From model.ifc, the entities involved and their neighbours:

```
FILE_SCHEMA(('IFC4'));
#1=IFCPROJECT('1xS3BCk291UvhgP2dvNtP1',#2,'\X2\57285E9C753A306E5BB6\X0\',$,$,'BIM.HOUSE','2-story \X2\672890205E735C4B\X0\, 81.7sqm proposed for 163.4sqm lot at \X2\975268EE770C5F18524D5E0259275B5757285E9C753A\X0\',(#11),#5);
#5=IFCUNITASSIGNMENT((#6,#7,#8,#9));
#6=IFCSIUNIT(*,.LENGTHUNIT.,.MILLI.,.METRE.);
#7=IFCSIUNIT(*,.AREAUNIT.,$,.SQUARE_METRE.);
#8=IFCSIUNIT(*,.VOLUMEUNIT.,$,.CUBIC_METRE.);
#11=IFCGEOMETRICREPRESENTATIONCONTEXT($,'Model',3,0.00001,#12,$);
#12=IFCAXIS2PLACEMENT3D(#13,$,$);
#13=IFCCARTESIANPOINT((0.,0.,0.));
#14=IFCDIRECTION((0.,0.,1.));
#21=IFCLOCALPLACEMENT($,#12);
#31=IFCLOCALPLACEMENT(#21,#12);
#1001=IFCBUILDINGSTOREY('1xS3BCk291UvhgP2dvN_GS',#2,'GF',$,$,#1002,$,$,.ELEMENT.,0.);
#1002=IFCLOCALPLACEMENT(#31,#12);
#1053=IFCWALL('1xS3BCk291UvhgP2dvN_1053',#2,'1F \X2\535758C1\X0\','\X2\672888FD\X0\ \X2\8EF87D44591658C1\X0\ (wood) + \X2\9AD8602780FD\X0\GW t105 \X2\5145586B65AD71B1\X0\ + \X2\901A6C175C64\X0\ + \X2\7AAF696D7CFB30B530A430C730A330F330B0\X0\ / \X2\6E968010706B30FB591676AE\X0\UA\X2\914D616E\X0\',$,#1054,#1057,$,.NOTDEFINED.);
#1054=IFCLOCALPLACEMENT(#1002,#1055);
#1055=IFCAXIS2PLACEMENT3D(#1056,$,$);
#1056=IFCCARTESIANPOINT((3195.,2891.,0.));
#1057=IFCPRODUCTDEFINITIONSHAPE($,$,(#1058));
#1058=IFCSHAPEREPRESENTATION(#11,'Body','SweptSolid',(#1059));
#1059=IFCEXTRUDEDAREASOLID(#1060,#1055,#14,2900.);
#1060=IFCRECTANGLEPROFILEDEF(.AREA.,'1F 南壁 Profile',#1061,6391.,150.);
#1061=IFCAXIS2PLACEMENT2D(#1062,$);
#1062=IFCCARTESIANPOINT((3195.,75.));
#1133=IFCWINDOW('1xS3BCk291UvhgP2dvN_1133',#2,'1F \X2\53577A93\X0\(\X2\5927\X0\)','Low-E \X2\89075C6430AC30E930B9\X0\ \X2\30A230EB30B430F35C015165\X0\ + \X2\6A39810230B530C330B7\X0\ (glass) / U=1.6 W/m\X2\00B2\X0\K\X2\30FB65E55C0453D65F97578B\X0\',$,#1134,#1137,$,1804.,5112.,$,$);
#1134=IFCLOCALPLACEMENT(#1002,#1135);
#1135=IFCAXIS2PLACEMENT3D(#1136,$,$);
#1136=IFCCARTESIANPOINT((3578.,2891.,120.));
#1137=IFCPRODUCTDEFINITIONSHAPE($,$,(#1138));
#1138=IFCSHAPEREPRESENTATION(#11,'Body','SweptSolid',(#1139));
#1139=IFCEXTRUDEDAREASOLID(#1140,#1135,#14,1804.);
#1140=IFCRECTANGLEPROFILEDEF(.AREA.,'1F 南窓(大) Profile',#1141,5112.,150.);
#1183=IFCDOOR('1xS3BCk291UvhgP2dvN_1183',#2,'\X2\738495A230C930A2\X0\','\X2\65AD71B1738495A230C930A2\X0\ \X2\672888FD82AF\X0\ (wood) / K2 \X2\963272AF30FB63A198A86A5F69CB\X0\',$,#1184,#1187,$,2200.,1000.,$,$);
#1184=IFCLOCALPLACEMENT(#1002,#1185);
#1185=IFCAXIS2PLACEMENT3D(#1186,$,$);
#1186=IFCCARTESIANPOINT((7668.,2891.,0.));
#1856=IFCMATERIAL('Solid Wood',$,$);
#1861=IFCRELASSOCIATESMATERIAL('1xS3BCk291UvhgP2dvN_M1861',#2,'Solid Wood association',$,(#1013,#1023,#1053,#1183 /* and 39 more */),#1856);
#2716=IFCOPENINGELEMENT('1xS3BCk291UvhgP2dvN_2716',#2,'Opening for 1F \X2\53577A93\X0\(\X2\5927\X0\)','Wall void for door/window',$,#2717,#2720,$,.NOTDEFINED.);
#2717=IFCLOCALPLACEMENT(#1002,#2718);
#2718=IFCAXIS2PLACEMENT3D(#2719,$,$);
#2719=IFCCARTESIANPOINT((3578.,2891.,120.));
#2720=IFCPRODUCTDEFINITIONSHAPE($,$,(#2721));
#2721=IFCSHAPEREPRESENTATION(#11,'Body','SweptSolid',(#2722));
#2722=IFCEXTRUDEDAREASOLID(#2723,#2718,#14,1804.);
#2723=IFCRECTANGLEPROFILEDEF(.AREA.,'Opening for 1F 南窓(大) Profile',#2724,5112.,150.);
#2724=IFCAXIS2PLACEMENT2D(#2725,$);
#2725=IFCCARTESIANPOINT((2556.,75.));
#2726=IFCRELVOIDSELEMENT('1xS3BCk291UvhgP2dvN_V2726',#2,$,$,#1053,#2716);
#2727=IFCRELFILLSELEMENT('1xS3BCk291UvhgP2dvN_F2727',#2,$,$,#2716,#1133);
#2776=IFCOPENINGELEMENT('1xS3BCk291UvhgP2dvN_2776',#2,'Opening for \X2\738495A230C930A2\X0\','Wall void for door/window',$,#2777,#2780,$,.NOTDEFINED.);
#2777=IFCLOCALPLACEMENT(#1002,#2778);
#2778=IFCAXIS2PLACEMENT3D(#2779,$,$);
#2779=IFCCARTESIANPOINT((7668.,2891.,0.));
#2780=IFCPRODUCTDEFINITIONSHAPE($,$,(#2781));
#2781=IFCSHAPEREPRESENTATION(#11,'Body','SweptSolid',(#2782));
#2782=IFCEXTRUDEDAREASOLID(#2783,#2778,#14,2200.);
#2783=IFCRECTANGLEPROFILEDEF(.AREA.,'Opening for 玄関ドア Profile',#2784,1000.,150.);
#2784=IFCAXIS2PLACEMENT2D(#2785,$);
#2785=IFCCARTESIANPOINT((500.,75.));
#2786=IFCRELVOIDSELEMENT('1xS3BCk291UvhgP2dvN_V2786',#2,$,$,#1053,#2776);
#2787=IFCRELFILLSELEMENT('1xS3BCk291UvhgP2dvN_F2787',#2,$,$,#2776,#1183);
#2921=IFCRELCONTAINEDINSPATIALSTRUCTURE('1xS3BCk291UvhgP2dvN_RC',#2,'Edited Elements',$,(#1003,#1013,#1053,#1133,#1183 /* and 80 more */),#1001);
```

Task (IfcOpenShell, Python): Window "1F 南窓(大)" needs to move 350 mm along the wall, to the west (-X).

```python
import ifcopenshell
import ifcopenshell.api.geometry
import ifcopenshell.util.placement
import ifcopenshell.util.unit

model = ifcopenshell.open("model.ifc")
unit_scale = ifcopenshell.util.unit.calculate_unit_scale(model)

window = model.by_guid("1xS3BCk291UvhgP2dvN_1133")
opening = window.FillsVoids[0].RelatingOpeningElement
wall = opening.VoidsElements[0].RelatingBuildingElement

wall_matrix = ifcopenshell.util.placement.get_local_placement(wall.ObjectPlacement)
shift = wall_matrix[:3, 0] * -0.35 / unit_scale
before = ifcopenshell.util.placement.get_local_placement(window.ObjectPlacement)[:3, 3].copy()

# The window is not placed relative to its opening, so move both.
for product in (opening, window):
    matrix = ifcopenshell.util.placement.get_local_placement(product.ObjectPlacement)
    matrix[:3, 3] += shift
    ifcopenshell.api.geometry.edit_object_placement(model, product=product, matrix=matrix, is_si=False)

after = ifcopenshell.util.placement.get_local_placement(window.ObjectPlacement)[:3, 3]
print("window moved by", (after - before).round(3) + 0.0)

model.write("model_edited.ifc")
```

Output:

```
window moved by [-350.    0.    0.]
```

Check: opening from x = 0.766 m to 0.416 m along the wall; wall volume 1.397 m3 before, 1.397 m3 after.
